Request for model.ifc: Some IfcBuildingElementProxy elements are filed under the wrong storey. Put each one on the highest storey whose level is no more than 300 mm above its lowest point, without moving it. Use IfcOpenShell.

First a look at what the model holds.

```python
import ifcopenshell
import ifcopenshell.util.element
import ifcopenshell.util.placement

model = ifcopenshell.open("model.ifc")
print(model.schema)
for storey in model.by_type("IfcBuildingStorey"):
    level = ifcopenshell.util.placement.get_storey_elevation(storey)
    count = sum(e.is_a("IfcBuildingElementProxy") for e in ifcopenshell.util.element.get_contained(storey))
    print(storey.id(), storey.Name, round(level, 3), count, sep=" | ")
```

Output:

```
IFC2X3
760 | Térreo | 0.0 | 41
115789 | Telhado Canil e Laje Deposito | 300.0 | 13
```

```python
import ifcopenshell
import ifcopenshell.api.spatial
import ifcopenshell.geom
import ifcopenshell.util.element
import ifcopenshell.util.placement
import ifcopenshell.util.shape
import ifcopenshell.util.unit

model = ifcopenshell.open("model.ifc")
unit_scale = ifcopenshell.util.unit.calculate_unit_scale(model)
settings = ifcopenshell.geom.settings()

levels = sorted(
    ((ifcopenshell.util.placement.get_storey_elevation(s) * unit_scale, s) for s in model.by_type("IfcBuildingStorey")),
    key=lambda pair: pair[0],
)

for e in model.by_type("IfcBuildingElementProxy"):
    current = e.ContainedInStructure[0].RelatingStructure if e.ContainedInStructure else None
    if current is None or not current.is_a("IfcBuildingStorey"):
        continue
    shape = ifcopenshell.geom.create_shape(settings, e)
    bottom = ifcopenshell.util.shape.get_shape_bottom_elevation(shape, shape.geometry)
    below = [s for level, s in levels if level <= bottom + 0.3]
    storey = below[-1] if below else levels[0][1]
    if storey != current:
        # assign_container keeps the world position.
        ifcopenshell.api.spatial.assign_container(model, products=[e], relating_structure=storey)
        print(e.id(), current.Name, "->", storey.Name)

model.write("model_updated.ifc")
```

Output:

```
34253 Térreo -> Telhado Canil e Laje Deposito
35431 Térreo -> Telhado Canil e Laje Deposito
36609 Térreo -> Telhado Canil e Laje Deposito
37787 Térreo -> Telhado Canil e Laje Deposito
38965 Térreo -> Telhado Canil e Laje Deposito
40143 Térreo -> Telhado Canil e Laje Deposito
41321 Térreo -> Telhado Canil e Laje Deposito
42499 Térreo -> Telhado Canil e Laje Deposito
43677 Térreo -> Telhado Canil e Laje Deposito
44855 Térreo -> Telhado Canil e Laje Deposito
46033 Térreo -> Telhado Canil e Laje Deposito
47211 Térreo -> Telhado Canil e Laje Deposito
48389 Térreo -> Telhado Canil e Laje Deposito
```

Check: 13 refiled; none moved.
